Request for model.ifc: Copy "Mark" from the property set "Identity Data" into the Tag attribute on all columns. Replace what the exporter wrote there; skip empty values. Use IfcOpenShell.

First a look at what the model holds.

```python
import ifcopenshell
import ifcopenshell.util.element

model = ifcopenshell.open("model.ifc")
print(model.schema)
columns = model.by_type("IfcColumn")
print(len(columns), "columns")
for e in columns[:8]:
    source = ifcopenshell.util.element.get_pset(e, "Identity Data", "Mark")
    target = e.Tag
    print(e.id(), repr(source), repr(target), sep=" | ")
```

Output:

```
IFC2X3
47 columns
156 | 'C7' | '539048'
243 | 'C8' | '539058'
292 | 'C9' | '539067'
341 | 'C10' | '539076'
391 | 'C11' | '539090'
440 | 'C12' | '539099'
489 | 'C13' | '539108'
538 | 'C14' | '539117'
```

```python
import ifcopenshell
import ifcopenshell.util.element

model = ifcopenshell.open("model.ifc")

count = 0
for e in model.by_type("IfcColumn"):
    value = ifcopenshell.util.element.get_pset(e, "Identity Data", "Mark")
    current = e.Tag
    if not value or not value.strip() or current == value:
        continue
    e.Tag = value
    count += 1

print(count, "columns updated")

model.write("model_edited.ifc")
```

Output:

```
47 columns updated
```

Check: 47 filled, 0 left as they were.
